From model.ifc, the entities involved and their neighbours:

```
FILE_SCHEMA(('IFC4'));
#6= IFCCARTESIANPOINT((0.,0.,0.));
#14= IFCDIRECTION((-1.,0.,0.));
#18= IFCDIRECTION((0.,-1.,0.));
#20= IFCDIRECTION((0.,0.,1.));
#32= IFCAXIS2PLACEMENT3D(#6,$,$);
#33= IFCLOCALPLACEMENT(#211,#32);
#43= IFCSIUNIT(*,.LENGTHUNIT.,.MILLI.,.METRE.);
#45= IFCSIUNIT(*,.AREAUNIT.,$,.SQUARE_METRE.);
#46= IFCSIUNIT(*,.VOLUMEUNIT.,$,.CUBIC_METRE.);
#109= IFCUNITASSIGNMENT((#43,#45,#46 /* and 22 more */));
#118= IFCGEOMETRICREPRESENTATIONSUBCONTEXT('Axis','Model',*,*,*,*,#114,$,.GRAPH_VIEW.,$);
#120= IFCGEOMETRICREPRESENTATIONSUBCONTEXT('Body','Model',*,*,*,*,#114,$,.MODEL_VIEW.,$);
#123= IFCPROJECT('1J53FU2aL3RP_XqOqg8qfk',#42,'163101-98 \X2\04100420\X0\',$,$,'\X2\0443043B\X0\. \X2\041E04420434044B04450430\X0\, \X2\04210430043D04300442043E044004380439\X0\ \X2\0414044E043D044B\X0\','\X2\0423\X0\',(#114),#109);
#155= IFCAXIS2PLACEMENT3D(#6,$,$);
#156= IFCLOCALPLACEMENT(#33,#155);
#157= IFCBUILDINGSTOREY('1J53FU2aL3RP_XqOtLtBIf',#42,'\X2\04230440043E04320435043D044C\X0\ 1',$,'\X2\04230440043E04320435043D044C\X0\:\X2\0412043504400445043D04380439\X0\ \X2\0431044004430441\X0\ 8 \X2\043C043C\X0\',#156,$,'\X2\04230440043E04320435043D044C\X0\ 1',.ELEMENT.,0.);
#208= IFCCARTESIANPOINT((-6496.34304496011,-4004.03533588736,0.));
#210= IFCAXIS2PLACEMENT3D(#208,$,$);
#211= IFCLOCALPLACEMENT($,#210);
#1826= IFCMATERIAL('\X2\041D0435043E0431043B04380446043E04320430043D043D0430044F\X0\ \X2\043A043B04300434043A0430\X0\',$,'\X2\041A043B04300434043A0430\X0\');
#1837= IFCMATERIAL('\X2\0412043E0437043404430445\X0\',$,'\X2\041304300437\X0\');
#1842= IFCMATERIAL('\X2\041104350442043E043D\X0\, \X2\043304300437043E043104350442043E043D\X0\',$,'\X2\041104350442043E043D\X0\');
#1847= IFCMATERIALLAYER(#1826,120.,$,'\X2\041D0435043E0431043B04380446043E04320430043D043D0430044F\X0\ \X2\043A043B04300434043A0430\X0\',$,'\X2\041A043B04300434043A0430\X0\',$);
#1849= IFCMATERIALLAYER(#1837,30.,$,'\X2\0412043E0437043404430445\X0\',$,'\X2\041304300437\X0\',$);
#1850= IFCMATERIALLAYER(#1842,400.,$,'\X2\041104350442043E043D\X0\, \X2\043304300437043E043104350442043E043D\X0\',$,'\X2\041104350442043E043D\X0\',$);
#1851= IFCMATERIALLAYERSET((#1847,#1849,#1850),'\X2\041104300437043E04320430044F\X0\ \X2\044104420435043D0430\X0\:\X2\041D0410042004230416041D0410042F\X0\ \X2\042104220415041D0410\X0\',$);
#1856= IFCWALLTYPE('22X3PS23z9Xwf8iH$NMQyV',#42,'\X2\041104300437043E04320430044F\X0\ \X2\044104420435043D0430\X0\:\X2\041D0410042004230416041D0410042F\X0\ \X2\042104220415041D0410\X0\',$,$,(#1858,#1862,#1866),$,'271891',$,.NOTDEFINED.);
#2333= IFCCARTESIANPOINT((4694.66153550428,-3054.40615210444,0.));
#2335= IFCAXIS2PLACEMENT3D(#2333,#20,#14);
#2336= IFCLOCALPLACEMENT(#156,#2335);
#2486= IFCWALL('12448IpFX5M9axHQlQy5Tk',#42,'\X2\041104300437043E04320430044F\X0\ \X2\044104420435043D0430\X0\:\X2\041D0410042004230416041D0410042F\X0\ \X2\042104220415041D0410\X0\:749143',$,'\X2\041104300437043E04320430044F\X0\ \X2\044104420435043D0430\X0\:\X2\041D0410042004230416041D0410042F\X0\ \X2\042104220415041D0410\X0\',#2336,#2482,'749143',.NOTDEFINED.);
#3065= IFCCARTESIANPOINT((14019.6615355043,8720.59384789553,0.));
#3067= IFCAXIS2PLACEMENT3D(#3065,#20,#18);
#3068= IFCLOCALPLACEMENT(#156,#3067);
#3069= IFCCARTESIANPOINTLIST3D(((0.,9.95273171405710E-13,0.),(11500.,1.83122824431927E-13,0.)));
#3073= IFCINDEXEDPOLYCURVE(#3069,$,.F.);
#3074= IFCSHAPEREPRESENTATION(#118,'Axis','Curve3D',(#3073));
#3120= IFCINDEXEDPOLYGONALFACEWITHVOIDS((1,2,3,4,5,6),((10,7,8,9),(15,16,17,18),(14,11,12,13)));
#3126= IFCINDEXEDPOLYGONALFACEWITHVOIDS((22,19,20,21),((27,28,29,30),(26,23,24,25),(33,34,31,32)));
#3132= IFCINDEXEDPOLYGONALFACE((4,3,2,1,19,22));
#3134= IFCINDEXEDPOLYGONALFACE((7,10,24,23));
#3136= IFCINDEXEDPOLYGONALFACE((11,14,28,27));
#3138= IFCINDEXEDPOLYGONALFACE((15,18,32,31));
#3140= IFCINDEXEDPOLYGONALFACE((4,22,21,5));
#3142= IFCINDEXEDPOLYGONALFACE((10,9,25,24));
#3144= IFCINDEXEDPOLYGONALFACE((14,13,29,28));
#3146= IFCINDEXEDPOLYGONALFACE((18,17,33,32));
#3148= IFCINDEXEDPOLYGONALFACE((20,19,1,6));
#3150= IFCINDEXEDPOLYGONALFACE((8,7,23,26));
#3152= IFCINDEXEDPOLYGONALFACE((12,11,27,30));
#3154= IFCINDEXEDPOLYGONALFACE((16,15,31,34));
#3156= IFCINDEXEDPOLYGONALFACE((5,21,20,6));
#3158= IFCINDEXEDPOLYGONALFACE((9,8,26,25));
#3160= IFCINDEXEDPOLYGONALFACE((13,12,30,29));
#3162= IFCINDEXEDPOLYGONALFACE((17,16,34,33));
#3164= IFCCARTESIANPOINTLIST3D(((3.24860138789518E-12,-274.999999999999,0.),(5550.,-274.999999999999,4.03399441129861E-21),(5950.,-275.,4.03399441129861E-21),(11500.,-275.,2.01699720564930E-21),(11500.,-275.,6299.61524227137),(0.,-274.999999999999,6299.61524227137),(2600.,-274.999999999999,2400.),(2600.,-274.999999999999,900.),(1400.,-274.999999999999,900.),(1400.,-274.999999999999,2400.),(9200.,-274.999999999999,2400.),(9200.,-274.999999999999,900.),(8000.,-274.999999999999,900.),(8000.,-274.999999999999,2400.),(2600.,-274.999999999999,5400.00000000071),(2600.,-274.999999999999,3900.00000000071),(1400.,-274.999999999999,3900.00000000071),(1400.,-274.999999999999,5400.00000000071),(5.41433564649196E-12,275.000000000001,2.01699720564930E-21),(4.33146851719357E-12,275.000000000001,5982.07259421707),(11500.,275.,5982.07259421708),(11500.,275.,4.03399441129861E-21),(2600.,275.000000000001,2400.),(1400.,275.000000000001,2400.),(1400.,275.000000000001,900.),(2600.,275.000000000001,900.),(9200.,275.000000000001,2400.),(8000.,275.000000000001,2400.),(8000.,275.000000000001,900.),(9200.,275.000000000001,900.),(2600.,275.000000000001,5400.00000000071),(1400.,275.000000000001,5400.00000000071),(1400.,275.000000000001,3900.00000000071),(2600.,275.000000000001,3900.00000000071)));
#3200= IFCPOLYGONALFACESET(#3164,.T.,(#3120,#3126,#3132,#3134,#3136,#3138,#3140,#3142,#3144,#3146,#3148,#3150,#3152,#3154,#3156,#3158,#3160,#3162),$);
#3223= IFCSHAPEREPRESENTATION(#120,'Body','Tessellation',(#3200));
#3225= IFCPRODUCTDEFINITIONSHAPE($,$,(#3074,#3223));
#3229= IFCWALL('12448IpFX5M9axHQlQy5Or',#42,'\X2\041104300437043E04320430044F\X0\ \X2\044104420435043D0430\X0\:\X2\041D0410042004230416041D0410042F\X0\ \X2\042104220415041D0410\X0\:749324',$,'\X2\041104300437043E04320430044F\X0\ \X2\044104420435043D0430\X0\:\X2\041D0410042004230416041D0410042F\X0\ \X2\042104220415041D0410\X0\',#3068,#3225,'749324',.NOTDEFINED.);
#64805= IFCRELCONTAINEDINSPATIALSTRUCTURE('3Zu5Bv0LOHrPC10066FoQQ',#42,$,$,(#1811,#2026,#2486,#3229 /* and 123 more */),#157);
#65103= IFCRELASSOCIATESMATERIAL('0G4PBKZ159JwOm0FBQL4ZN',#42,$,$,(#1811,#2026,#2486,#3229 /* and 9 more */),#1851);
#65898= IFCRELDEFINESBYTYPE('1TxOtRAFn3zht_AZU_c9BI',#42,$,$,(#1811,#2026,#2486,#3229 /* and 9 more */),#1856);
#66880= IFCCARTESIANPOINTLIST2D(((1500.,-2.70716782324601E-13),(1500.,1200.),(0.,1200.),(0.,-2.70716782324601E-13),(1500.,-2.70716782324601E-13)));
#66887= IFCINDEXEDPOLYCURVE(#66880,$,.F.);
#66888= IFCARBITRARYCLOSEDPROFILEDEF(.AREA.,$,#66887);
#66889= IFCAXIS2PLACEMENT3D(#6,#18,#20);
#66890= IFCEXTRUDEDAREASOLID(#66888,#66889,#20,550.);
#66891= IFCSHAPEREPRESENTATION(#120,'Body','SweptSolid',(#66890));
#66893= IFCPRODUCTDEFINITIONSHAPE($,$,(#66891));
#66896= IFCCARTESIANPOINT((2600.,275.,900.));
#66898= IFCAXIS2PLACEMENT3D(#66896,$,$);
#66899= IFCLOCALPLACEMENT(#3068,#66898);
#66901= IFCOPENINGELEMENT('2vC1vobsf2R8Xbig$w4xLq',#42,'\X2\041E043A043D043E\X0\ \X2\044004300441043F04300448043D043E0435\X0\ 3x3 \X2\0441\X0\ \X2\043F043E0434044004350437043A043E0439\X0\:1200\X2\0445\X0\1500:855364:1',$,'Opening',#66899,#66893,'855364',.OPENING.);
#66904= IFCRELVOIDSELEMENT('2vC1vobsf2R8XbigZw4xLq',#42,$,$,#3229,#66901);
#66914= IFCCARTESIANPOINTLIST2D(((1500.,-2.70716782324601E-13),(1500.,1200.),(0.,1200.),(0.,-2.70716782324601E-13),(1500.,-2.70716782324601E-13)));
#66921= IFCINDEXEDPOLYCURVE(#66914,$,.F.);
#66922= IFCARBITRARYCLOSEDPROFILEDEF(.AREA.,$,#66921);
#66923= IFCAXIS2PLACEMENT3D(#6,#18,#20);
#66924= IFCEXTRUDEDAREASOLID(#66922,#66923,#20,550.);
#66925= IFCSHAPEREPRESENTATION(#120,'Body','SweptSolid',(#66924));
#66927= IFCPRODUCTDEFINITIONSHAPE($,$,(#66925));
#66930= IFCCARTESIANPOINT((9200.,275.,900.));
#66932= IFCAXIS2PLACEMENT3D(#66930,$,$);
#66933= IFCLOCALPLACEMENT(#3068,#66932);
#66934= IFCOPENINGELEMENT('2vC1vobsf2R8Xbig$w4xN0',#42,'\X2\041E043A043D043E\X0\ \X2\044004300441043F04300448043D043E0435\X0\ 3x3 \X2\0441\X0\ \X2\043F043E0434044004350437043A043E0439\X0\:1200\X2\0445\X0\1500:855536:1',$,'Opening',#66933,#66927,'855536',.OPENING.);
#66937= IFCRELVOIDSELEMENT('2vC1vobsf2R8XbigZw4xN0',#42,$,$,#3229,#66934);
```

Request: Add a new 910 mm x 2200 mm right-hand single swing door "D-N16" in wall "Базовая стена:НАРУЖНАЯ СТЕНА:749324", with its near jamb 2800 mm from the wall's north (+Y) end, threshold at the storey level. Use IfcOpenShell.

```python
import numpy as np
import ifcopenshell
import ifcopenshell.api.feature
import ifcopenshell.api.geometry
import ifcopenshell.api.root
import ifcopenshell.api.spatial
import ifcopenshell.geom
import ifcopenshell.util.element
import ifcopenshell.util.placement
import ifcopenshell.util.representation
import ifcopenshell.util.shape
import ifcopenshell.util.unit

model = ifcopenshell.open("model.ifc")
unit_scale = ifcopenshell.util.unit.calculate_unit_scale(model)
settings = ifcopenshell.geom.settings()


def volume(element):
    """Net volume in cubic metres, openings subtracted."""
    shape = ifcopenshell.geom.create_shape(settings, element)
    return ifcopenshell.util.shape.get_volume(shape.geometry)


wall = model.by_guid("12448IpFX5M9axHQlQy5Or")
storey = ifcopenshell.util.element.get_container(wall, ifc_class="IfcBuildingStorey")
context = ifcopenshell.util.representation.get_context(model, "Model", "Body", "MODEL_VIEW")
before = volume(wall)

width, height, from_end, sill = 0.91, 2.2, 2.8, 0.0  # metres

# The wall runs along its own X axis, and the end named is its -X end.
wall_shape = ifcopenshell.geom.create_shape(settings, wall)
x, y, z = ifcopenshell.util.shape.get_vertices(wall_shape.geometry).T
start = x.min() + from_end
face, thickness = float(y.min()), float(y.max() - y.min())
wall_matrix = ifcopenshell.util.placement.get_local_placement(wall.ObjectPlacement)
level = ifcopenshell.util.placement.get_local_placement(storey.ObjectPlacement)[2, 3]


def in_wall(x, y):
    """Placement at x, y metres in the wall's axes, at sill height."""
    matrix = wall_matrix.copy()
    matrix[:, 3] = wall_matrix @ np.array([x / unit_scale, y / unit_scale, 0.0, 1.0])
    matrix[2, 3] = level + sill / unit_scale
    return matrix


# Opening: a box that overshoots both wall faces by 50 mm.
opening = ifcopenshell.api.root.create_entity(model, ifc_class="IfcOpeningElement", predefined_type="OPENING")
box = ifcopenshell.api.geometry.add_wall_representation(
    model, context=context, length=width, height=height, thickness=thickness + 0.1
)
ifcopenshell.api.geometry.assign_representation(model, product=opening, representation=box)
ifcopenshell.api.geometry.edit_object_placement(model, product=opening, matrix=in_wall(start, face - 0.05), is_si=False)
ifcopenshell.api.feature.add_feature(model, feature=opening, element=wall)

door = ifcopenshell.api.root.create_entity(model, ifc_class="IfcDoor", name="D-N16", predefined_type="DOOR")
door.OverallWidth, door.OverallHeight = width / unit_scale, height / unit_scale
door.OperationType = "SINGLE_SWING_RIGHT"
body = ifcopenshell.api.geometry.add_door_representation(
    model,
    context=context,
    overall_width=door.OverallWidth,
    overall_height=door.OverallHeight,
    operation_type="SINGLE_SWING_RIGHT",
    lining_properties={"LiningDepth": thickness / unit_scale, "ThresholdDepth": thickness / unit_scale},
)
ifcopenshell.api.geometry.assign_representation(model, product=door, representation=body)
ifcopenshell.api.spatial.assign_container(model, products=[door], relating_structure=storey)
ifcopenshell.api.feature.add_filling(model, opening=opening, element=door)

# The lining spans the wall, so the door starts at the wall face.
ifcopenshell.api.geometry.edit_object_placement(model, product=door, matrix=in_wall(start, face), is_si=False)

after = volume(wall)

print(f"wall volume {before:.3f} -> {after:.3f} m3")

model.write("model_updated.ifc")
```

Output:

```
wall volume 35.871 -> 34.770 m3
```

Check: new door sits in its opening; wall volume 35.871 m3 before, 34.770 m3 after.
